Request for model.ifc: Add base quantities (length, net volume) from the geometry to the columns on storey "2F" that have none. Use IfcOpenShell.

First a look at what the model holds.

```python
import ifcopenshell
import ifcopenshell.util.element
import ifcopenshell.util.unit

model = ifcopenshell.open("model.ifc")
print(model.schema)
for unit_type in ("LENGTHUNIT", "AREAUNIT", "VOLUMEUNIT"):
    print(unit_type, ifcopenshell.util.unit.calculate_unit_scale(model, unit_type))
storey = next(s for s in model.by_type("IfcBuildingStorey") if s.Name == "2F")
columns = [e for e in ifcopenshell.util.element.get_decomposition(storey) if e.is_a("IfcColumn")]
for e in sorted(columns, key=lambda e: e.id()):
    print(e.id(), e.is_a(), e.Name, list(ifcopenshell.util.element.get_psets(e, qtos_only=True)), sep=" | ")
```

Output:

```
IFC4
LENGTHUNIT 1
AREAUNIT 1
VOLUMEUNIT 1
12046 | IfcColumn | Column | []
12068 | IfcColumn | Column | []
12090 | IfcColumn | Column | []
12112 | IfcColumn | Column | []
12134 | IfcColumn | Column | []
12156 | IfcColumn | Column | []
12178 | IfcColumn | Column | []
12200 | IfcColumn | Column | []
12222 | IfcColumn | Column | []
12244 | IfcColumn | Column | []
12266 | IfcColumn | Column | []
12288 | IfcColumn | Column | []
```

```python
import ifcopenshell
import ifcopenshell.api.pset
import ifcopenshell.geom
import ifcopenshell.util.element
import ifcopenshell.util.shape
import ifcopenshell.util.unit

model = ifcopenshell.open("model.ifc")
unit_scale = ifcopenshell.util.unit.calculate_unit_scale(model)
volume_scale = ifcopenshell.util.unit.calculate_unit_scale(model, "VOLUMEUNIT")
settings = ifcopenshell.geom.settings()

storey = next(s for s in model.by_type("IfcBuildingStorey") if s.Name == "2F")
columns = [e for e in ifcopenshell.util.element.get_decomposition(storey) if e.is_a("IfcColumn")]

for e in sorted(columns, key=lambda e: e.id()):
    if ifcopenshell.util.element.get_psets(e, qtos_only=True, should_inherit=False):
        continue
    # Geometry comes back in metres, in the element's own axes.
    shape = ifcopenshell.geom.create_shape(settings, e)
    values = {
        "Length": ifcopenshell.util.shape.get_z(shape.geometry) / unit_scale,
        "NetVolume": ifcopenshell.util.shape.get_volume(shape.geometry) / volume_scale,
    }
    qto = ifcopenshell.api.pset.add_qto(model, product=e, name="Qto_ColumnBaseQuantities")
    ifcopenshell.api.pset.edit_qto(model, qto=qto, properties=values)
    print(e.id(), {k: round(v, 3) for k, v in values.items()})

model.write("model_v2.ifc")
```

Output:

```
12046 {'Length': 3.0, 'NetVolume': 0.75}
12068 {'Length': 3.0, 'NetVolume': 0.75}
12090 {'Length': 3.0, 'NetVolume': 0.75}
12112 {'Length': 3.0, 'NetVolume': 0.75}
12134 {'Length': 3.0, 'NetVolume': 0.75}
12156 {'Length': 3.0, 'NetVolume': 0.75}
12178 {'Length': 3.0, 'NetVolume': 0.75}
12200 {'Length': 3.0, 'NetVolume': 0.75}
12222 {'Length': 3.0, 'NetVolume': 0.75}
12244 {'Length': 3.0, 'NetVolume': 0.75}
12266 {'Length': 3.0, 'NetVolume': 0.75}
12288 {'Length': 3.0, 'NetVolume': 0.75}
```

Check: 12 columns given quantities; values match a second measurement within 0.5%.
